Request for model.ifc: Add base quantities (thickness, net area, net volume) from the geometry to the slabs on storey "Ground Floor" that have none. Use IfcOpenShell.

First a look at what the model holds.

```python
import ifcopenshell
import ifcopenshell.util.element
import ifcopenshell.util.unit

model = ifcopenshell.open("model.ifc")
print(model.schema)
for unit_type in ("LENGTHUNIT", "AREAUNIT", "VOLUMEUNIT"):
    print(unit_type, ifcopenshell.util.unit.calculate_unit_scale(model, unit_type))
storey = next(s for s in model.by_type("IfcBuildingStorey") if s.Name == "Ground Floor")
slabs = [e for e in ifcopenshell.util.element.get_decomposition(storey) if e.is_a("IfcSlab")]
for e in sorted(slabs, key=lambda e: e.id()):
    print(e.id(), e.is_a(), e.Name, list(ifcopenshell.util.element.get_psets(e, qtos_only=True)), sep=" | ")
```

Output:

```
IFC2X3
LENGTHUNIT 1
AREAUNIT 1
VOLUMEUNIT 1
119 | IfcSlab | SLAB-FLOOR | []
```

```python
import ifcopenshell
import ifcopenshell.api.pset
import ifcopenshell.geom
import ifcopenshell.util.element
import ifcopenshell.util.shape
import ifcopenshell.util.unit

model = ifcopenshell.open("model.ifc")
unit_scale = ifcopenshell.util.unit.calculate_unit_scale(model)
area_scale = ifcopenshell.util.unit.calculate_unit_scale(model, "AREAUNIT")
volume_scale = ifcopenshell.util.unit.calculate_unit_scale(model, "VOLUMEUNIT")
settings = ifcopenshell.geom.settings()

storey = next(s for s in model.by_type("IfcBuildingStorey") if s.Name == "Ground Floor")
slabs = [e for e in ifcopenshell.util.element.get_decomposition(storey) if e.is_a("IfcSlab")]

for e in sorted(slabs, key=lambda e: e.id()):
    if ifcopenshell.util.element.get_psets(e, qtos_only=True, should_inherit=False):
        continue
    # Geometry comes back in metres, in the element's own axes.
    shape = ifcopenshell.geom.create_shape(settings, e)
    values = {
        "Width": ifcopenshell.util.shape.get_z(shape.geometry) / unit_scale,
        "NetArea": ifcopenshell.util.shape.get_footprint_area(shape.geometry) / area_scale,
        "NetVolume": ifcopenshell.util.shape.get_volume(shape.geometry) / volume_scale,
    }
    qto = ifcopenshell.api.pset.add_qto(model, product=e, name="BaseQuantities")
    ifcopenshell.api.pset.edit_qto(model, qto=qto, properties=values)
    print(e.id(), {k: round(v, 3) for k, v in values.items()})

model.write("model-out.ifc")
```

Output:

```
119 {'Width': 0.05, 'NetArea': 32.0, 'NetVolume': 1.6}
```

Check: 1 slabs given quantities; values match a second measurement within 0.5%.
